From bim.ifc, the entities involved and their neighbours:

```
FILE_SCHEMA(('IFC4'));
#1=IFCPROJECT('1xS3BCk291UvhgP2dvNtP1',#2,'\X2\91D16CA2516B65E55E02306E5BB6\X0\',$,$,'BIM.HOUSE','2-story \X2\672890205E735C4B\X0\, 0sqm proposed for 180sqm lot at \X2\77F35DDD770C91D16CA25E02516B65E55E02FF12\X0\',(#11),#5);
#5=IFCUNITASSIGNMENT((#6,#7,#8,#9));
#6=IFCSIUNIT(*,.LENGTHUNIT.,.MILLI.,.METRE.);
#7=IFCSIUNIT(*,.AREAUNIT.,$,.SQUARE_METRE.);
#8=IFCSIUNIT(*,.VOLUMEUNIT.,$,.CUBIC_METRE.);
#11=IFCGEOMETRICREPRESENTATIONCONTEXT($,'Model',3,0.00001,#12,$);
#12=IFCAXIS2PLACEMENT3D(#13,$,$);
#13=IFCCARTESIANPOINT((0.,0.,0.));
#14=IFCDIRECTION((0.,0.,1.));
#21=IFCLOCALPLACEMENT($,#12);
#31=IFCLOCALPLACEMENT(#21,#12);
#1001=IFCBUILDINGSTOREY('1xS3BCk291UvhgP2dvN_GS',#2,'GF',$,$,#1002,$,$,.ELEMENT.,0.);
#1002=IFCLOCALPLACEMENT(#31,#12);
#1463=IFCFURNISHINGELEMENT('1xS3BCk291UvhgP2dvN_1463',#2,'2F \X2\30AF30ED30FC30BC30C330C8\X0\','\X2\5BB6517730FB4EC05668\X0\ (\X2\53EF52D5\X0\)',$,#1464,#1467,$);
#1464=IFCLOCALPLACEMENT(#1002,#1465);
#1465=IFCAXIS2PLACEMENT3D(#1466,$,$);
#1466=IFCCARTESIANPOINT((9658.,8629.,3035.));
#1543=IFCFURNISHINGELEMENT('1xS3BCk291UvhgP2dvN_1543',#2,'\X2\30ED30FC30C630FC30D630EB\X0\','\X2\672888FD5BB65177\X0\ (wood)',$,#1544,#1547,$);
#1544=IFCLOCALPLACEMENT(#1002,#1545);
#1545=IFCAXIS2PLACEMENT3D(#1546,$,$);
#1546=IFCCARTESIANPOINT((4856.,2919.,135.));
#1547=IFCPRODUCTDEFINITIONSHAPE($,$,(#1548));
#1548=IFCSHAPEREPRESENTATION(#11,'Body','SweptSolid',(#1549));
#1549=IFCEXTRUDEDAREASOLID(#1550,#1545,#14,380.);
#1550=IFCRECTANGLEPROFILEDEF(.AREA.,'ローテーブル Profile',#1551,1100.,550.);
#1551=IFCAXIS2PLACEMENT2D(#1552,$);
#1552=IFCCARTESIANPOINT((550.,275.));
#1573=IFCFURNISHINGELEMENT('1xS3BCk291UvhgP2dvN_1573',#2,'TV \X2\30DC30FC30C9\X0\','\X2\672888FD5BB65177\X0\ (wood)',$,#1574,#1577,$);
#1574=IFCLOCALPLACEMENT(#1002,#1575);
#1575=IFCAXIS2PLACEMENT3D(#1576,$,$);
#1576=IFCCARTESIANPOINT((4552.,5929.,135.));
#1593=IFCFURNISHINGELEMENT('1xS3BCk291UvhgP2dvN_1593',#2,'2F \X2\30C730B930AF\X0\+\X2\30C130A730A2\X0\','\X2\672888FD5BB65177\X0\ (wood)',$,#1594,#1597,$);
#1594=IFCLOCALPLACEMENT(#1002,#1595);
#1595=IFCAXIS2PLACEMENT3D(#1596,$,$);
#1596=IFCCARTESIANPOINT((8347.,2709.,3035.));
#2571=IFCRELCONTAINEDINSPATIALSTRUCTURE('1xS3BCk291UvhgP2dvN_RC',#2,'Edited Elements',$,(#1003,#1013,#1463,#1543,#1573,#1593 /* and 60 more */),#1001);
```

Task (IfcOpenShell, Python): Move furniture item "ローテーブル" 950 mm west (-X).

```python
import ifcopenshell
import ifcopenshell.api.geometry
import ifcopenshell.util.placement
import ifcopenshell.util.unit

model = ifcopenshell.open("bim.ifc")
unit_scale = ifcopenshell.util.unit.calculate_unit_scale(model)

item = model.by_guid("1xS3BCk291UvhgP2dvN_1543")
matrix = ifcopenshell.util.placement.get_local_placement(item.ObjectPlacement)
matrix[0, 3] -= 0.95 / unit_scale
ifcopenshell.api.geometry.edit_object_placement(model, product=item, matrix=matrix, is_si=False)

print(ifcopenshell.util.placement.get_local_placement(item.ObjectPlacement).round(3) + 0.0)

model.write("bim_edited.ifc")
```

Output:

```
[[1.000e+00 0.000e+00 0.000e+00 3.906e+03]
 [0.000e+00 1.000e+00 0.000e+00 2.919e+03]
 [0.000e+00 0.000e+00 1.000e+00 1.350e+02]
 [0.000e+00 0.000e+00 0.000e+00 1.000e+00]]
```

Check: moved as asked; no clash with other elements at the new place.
